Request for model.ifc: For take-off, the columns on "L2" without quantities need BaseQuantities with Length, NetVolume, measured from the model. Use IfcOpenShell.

First a look at what the model holds.

```python
import ifcopenshell
import ifcopenshell.util.element
import ifcopenshell.util.unit

model = ifcopenshell.open("model.ifc")
print(model.schema)
for unit_type in ("LENGTHUNIT", "AREAUNIT", "VOLUMEUNIT"):
    print(unit_type, ifcopenshell.util.unit.calculate_unit_scale(model, unit_type))
storey = next(s for s in model.by_type("IfcBuildingStorey") if s.Name == "L2")
columns = [e for e in ifcopenshell.util.element.get_decomposition(storey) if e.is_a("IfcColumn")]
for e in sorted(columns, key=lambda e: e.id()):
    print(e.id(), e.is_a(), e.Name, list(ifcopenshell.util.element.get_psets(e, qtos_only=True)), sep=" | ")
```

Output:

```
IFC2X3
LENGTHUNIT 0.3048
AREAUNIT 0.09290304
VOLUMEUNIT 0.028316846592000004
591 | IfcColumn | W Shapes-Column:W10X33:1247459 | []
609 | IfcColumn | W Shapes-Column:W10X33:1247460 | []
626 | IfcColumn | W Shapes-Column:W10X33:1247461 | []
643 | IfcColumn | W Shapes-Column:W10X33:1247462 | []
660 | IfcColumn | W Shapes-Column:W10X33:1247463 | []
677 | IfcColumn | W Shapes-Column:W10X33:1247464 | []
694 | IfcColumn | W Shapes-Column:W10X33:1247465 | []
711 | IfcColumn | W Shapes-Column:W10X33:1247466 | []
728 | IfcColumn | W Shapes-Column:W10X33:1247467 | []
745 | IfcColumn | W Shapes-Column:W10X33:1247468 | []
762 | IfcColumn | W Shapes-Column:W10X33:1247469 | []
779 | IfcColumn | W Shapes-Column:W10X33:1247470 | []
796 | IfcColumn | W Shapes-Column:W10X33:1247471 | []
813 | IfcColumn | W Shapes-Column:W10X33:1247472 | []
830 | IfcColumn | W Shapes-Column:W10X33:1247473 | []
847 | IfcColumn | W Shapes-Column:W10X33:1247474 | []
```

```python
import ifcopenshell
import ifcopenshell.api.pset
import ifcopenshell.geom
import ifcopenshell.util.element
import ifcopenshell.util.shape
import ifcopenshell.util.unit

model = ifcopenshell.open("model.ifc")
unit_scale = ifcopenshell.util.unit.calculate_unit_scale(model)
volume_scale = ifcopenshell.util.unit.calculate_unit_scale(model, "VOLUMEUNIT")
settings = ifcopenshell.geom.settings()

storey = next(s for s in model.by_type("IfcBuildingStorey") if s.Name == "L2")
columns = [e for e in ifcopenshell.util.element.get_decomposition(storey) if e.is_a("IfcColumn")]

for e in sorted(columns, key=lambda e: e.id()):
    if ifcopenshell.util.element.get_psets(e, qtos_only=True, should_inherit=False):
        continue
    # Geometry comes back in metres, in the element's own axes.
    shape = ifcopenshell.geom.create_shape(settings, e)
    values = {
        "Length": ifcopenshell.util.shape.get_z(shape.geometry) / unit_scale,
        "NetVolume": ifcopenshell.util.shape.get_volume(shape.geometry) / volume_scale,
    }
    qto = ifcopenshell.api.pset.add_qto(model, product=e, name="BaseQuantities")
    ifcopenshell.api.pset.edit_qto(model, qto=qto, properties=values)
    print(e.id(), {k: round(v, 3) for k, v in values.items()})

model.write("model_rev.ifc")
```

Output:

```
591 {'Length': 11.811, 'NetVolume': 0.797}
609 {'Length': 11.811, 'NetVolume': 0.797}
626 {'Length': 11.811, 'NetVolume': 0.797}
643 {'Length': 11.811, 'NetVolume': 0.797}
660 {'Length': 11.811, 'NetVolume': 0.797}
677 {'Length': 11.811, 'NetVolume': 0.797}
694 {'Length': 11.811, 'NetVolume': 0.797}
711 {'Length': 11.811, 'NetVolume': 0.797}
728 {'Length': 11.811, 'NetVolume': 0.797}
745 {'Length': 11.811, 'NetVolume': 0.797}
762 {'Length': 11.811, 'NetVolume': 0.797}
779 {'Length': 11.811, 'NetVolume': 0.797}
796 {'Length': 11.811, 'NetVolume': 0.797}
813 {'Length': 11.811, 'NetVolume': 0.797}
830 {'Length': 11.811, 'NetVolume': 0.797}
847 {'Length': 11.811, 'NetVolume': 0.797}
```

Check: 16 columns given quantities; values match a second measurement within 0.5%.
